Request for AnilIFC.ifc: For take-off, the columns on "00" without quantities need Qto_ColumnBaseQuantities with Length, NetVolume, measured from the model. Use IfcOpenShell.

First a look at what the model holds.

```python
import ifcopenshell
import ifcopenshell.util.element
import ifcopenshell.util.unit

model = ifcopenshell.open("AnilIFC.ifc")
print(model.schema)
for unit_type in ("LENGTHUNIT", "AREAUNIT", "VOLUMEUNIT"):
    print(unit_type, ifcopenshell.util.unit.calculate_unit_scale(model, unit_type))
storey = next(s for s in model.by_type("IfcBuildingStorey") if s.Name == "00")
columns = [e for e in ifcopenshell.util.element.get_decomposition(storey) if e.is_a("IfcColumn")]
for e in sorted(columns, key=lambda e: e.id()):
    print(e.id(), e.is_a(), e.Name, list(ifcopenshell.util.element.get_psets(e, qtos_only=True)), sep=" | ")
```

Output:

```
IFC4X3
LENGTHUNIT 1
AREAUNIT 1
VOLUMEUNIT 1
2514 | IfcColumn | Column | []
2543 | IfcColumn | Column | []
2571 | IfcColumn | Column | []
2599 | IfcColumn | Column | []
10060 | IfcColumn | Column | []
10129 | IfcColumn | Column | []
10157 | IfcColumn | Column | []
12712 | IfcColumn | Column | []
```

```python
import ifcopenshell
import ifcopenshell.api.pset
import ifcopenshell.geom
import ifcopenshell.util.element
import ifcopenshell.util.shape
import ifcopenshell.util.unit

model = ifcopenshell.open("AnilIFC.ifc")
unit_scale = ifcopenshell.util.unit.calculate_unit_scale(model)
volume_scale = ifcopenshell.util.unit.calculate_unit_scale(model, "VOLUMEUNIT")
settings = ifcopenshell.geom.settings()

storey = next(s for s in model.by_type("IfcBuildingStorey") if s.Name == "00")
columns = [e for e in ifcopenshell.util.element.get_decomposition(storey) if e.is_a("IfcColumn")]

for e in sorted(columns, key=lambda e: e.id()):
    if ifcopenshell.util.element.get_psets(e, qtos_only=True, should_inherit=False):
        continue
    # Geometry comes back in metres, in the element's own axes.
    shape = ifcopenshell.geom.create_shape(settings, e)
    values = {
        "Length": ifcopenshell.util.shape.get_z(shape.geometry) / unit_scale,
        "NetVolume": ifcopenshell.util.shape.get_volume(shape.geometry) / volume_scale,
    }
    qto = ifcopenshell.api.pset.add_qto(model, product=e, name="Qto_ColumnBaseQuantities")
    ifcopenshell.api.pset.edit_qto(model, qto=qto, properties=values)
    print(e.id(), {k: round(v, 3) for k, v in values.items()})

model.write("AnilIFC-out.ifc")
```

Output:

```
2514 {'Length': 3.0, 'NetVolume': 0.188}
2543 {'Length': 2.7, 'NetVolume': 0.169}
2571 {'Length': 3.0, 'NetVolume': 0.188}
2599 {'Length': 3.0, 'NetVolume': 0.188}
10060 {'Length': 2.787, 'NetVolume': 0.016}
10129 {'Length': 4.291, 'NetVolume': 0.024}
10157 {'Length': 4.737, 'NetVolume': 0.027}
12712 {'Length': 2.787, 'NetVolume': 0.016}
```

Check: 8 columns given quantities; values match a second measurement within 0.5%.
